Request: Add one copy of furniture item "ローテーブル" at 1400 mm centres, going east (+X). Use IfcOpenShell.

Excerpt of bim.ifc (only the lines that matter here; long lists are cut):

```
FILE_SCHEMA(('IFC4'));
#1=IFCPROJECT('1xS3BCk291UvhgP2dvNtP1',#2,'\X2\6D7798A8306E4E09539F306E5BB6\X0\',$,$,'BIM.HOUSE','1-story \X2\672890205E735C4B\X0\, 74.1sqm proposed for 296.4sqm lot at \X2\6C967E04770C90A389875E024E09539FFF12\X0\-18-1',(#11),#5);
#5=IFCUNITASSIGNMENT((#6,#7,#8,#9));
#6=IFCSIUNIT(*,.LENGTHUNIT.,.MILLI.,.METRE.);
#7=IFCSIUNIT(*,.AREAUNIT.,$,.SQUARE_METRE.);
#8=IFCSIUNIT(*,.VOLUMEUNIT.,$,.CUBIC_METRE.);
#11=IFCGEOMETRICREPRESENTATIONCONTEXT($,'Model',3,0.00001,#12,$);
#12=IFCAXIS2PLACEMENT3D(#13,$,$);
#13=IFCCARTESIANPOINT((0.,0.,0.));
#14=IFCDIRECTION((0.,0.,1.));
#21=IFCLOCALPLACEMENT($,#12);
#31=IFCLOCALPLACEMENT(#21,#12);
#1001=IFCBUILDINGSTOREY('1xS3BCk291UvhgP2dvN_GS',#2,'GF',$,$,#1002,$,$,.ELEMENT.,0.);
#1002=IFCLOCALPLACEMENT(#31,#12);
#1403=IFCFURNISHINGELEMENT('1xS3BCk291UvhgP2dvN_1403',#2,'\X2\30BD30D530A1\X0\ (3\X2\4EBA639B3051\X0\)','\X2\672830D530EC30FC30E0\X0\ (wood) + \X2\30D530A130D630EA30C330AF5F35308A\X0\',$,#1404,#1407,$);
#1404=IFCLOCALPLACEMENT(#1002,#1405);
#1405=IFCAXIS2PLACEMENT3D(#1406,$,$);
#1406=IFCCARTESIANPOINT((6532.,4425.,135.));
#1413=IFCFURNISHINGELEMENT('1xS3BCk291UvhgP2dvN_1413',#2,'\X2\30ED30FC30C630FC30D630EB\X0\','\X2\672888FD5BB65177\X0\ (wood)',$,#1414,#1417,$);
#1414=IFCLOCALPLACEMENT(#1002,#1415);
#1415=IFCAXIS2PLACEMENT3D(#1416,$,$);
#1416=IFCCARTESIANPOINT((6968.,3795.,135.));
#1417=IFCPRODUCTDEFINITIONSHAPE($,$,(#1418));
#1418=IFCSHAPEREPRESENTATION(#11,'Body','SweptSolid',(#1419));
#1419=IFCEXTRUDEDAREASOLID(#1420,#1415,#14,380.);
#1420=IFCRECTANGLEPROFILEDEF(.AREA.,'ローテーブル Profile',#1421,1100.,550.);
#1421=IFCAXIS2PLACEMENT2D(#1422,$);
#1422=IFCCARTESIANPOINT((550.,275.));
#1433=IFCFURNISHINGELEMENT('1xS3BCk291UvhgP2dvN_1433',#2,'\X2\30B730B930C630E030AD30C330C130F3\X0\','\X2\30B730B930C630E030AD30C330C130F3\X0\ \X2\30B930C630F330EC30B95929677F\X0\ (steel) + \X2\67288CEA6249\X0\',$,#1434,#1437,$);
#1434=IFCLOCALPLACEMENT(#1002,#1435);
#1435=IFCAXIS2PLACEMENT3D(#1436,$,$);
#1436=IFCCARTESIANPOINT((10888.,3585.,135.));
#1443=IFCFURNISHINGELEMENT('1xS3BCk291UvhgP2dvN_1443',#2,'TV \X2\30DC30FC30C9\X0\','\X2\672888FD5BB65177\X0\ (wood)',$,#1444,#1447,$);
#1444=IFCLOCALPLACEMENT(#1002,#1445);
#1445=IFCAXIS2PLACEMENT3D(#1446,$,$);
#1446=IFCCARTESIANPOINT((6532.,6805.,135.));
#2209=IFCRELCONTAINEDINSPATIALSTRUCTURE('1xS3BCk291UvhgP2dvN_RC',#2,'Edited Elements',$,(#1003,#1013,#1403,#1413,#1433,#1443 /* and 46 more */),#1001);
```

```python
import numpy as np
import ifcopenshell
import ifcopenshell.api.geometry
import ifcopenshell.api.root
import ifcopenshell.util.element
import ifcopenshell.util.placement
import ifcopenshell.util.unit

model = ifcopenshell.open("bim.ifc")
unit_scale = ifcopenshell.util.unit.calculate_unit_scale(model)


def reuse_history(source, copy):
    """copy_class also copies each property set's owner history, people and application; keep the originals."""
    for rel in copy.IsDefinedBy:
        if rel.is_a("IfcRelDefinesByProperties") and (history := rel.RelatingPropertyDefinition.OwnerHistory):
            rel.RelatingPropertyDefinition.OwnerHistory = source.OwnerHistory
            ifcopenshell.util.element.remove_deep2(model, history)


source = model.by_id(1413)
base = ifcopenshell.util.placement.get_local_placement(source.ObjectPlacement)
step = np.array([1.0, 0.0, 0.0]) * 1.4 / unit_scale

for i in range(1, 2):
    copy = ifcopenshell.api.root.copy_class(model, product=source)
    copy.Representation = ifcopenshell.util.element.copy_deep(
        model, source.Representation, exclude=["IfcGeometricRepresentationContext", "IfcRepresentationMap"]
    )
    reuse_history(source, copy)
    matrix = base.copy()
    matrix[:3, 3] += i * step
    print("added at", matrix[:3, 3].round(3) + 0.0)
    ifcopenshell.api.geometry.edit_object_placement(model, product=copy, matrix=matrix, is_si=False)

model.write("bim_updated.ifc")
```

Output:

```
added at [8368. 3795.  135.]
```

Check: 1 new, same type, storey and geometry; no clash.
